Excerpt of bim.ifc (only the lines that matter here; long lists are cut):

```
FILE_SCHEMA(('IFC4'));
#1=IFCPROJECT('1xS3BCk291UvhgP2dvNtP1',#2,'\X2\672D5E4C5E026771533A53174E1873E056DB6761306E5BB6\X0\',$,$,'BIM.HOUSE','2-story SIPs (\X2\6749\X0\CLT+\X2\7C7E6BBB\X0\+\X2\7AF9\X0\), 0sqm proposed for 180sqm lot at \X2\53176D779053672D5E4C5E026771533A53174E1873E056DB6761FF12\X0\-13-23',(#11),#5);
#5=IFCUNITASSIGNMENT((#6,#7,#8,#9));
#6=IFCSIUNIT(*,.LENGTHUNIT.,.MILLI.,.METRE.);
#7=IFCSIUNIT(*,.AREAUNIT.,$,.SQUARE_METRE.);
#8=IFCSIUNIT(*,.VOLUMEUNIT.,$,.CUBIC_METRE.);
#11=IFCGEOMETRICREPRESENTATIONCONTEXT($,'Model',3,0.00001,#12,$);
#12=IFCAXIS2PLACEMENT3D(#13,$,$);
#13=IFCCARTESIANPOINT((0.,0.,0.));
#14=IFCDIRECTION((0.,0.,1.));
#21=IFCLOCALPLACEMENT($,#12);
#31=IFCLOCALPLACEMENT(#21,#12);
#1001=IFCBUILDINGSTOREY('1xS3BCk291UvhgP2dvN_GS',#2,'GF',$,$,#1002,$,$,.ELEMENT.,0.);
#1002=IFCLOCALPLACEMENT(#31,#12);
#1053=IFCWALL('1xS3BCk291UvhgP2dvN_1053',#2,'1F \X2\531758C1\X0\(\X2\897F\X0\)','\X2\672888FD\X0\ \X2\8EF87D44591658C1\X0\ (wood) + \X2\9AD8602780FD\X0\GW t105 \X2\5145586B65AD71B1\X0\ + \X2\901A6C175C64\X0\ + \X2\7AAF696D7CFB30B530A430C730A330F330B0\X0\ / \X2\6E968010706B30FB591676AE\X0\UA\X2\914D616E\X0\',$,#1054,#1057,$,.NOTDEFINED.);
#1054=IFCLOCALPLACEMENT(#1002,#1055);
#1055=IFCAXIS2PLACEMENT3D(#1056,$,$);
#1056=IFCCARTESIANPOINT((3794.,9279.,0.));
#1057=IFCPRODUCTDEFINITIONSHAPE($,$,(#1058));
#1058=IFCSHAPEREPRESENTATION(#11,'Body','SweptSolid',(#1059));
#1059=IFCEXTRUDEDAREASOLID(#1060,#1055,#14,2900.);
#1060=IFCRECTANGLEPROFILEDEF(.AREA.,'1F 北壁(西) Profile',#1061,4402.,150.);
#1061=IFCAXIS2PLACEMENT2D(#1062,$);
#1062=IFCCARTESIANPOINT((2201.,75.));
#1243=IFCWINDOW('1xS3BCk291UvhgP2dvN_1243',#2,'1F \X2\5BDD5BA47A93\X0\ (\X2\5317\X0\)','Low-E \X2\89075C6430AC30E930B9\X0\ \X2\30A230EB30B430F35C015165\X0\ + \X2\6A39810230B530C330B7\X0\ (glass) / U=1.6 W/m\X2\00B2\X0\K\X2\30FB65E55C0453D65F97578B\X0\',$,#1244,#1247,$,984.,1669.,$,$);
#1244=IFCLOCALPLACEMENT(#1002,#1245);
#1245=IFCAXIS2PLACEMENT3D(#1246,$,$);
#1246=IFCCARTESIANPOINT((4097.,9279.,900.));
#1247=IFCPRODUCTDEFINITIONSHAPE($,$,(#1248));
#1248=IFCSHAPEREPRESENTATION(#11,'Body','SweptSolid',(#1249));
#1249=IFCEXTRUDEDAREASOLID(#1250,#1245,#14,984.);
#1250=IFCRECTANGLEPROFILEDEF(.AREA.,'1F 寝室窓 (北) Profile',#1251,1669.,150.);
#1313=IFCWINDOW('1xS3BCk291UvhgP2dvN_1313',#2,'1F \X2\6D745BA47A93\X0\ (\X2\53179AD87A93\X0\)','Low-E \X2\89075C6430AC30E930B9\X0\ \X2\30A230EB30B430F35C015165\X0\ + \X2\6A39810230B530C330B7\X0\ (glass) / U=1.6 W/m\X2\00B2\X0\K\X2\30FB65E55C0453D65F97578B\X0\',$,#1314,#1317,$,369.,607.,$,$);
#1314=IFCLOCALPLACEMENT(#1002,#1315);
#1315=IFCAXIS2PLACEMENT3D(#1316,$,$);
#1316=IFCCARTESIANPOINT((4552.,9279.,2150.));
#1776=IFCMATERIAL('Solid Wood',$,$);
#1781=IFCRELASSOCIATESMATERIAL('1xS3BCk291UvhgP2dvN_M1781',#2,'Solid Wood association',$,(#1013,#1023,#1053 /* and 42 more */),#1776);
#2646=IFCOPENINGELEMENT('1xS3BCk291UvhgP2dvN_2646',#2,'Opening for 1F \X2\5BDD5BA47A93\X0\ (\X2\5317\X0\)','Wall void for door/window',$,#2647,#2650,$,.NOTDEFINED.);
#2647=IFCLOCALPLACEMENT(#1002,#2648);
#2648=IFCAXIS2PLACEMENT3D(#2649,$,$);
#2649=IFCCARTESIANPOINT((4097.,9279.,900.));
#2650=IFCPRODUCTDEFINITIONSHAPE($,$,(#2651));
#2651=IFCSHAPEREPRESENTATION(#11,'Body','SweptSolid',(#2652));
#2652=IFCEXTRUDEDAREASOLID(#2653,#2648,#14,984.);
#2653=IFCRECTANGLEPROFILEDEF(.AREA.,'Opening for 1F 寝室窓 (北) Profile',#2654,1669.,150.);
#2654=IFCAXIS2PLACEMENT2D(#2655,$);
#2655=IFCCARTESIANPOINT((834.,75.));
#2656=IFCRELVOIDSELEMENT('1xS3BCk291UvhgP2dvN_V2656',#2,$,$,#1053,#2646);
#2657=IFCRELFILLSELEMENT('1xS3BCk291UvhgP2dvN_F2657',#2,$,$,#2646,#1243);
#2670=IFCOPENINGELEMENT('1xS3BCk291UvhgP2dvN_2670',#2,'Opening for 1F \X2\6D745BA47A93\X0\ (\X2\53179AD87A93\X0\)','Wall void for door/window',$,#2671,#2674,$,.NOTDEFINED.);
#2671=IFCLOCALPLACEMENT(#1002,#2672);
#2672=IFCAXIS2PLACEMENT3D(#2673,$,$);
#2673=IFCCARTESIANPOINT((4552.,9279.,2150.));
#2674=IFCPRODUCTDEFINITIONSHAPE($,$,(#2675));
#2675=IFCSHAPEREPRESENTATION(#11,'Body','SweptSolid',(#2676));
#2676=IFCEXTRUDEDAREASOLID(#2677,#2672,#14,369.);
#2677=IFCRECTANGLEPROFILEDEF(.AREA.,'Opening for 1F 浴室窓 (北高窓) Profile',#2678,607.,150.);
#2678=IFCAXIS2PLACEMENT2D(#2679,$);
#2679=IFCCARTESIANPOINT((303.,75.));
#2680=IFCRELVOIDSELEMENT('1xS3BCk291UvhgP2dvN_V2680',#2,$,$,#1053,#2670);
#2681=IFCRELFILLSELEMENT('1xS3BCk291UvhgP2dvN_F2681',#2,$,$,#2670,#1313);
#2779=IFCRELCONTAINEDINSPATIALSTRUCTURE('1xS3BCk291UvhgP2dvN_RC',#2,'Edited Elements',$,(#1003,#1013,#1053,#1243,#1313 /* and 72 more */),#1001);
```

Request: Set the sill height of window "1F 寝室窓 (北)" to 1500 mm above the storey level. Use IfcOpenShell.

```python
import numpy as np
import ifcopenshell
import ifcopenshell.api.geometry
import ifcopenshell.geom
import ifcopenshell.util.element
import ifcopenshell.util.placement
import ifcopenshell.util.shape
import ifcopenshell.util.unit

model = ifcopenshell.open("bim.ifc")
unit_scale = ifcopenshell.util.unit.calculate_unit_scale(model)

window = model.by_guid("1xS3BCk291UvhgP2dvN_1243")
opening = window.FillsVoids[0].RelatingOpeningElement
storey = ifcopenshell.util.element.get_container(window, ifc_class="IfcBuildingStorey")
level = ifcopenshell.util.placement.get_local_placement(storey.ObjectPlacement)[2, 3]

# The opening's origin need not be at the sill, so measure its lowest point.
shape = ifcopenshell.geom.create_shape(ifcopenshell.geom.settings(), opening)
bottom = ifcopenshell.util.shape.get_shape_bottom_elevation(shape, shape.geometry) / unit_scale
dz = level + 1500.0 - bottom

shift = np.array([0.0, 0.0, dz])
# The window is not placed relative to its opening, so move both.
for product in (opening, window):
    matrix = ifcopenshell.util.placement.get_local_placement(product.ObjectPlacement)
    matrix[:3, 3] += shift
    ifcopenshell.api.geometry.edit_object_placement(model, product=product, matrix=matrix, is_si=False)

print(f"moved by {dz * unit_scale:+.3f} m")

model.write("bim-out.ifc")
```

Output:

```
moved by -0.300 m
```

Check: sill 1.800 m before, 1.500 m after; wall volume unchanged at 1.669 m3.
